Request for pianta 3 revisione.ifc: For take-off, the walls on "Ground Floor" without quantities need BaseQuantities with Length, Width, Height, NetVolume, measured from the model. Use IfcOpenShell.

First a look at what the model holds.

```python
import ifcopenshell
import ifcopenshell.util.element
import ifcopenshell.util.unit

model = ifcopenshell.open("pianta 3 revisione.ifc")
print(model.schema)
for unit_type in ("LENGTHUNIT", "AREAUNIT", "VOLUMEUNIT"):
    print(unit_type, ifcopenshell.util.unit.calculate_unit_scale(model, unit_type))
storey = next(s for s in model.by_type("IfcBuildingStorey") if s.Name == "Ground Floor")
walls = [e for e in ifcopenshell.util.element.get_decomposition(storey) if e.is_a("IfcWall")]
for e in sorted(walls, key=lambda e: e.id()):
    print(e.id(), e.is_a(), e.Name, list(ifcopenshell.util.element.get_psets(e, qtos_only=True)), sep=" | ")
```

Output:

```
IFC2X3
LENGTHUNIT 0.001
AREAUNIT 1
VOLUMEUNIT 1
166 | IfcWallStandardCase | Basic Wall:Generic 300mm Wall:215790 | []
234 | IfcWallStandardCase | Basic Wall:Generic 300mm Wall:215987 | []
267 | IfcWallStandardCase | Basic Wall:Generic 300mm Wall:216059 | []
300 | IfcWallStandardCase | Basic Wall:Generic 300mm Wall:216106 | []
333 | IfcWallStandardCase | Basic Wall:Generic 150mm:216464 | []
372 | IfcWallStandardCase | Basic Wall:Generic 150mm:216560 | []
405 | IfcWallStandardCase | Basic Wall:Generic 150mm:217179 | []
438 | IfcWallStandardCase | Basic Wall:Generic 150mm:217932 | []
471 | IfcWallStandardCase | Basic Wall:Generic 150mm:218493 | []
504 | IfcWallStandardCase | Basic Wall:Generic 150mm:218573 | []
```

```python
import ifcopenshell
import ifcopenshell.api.pset
import ifcopenshell.geom
import ifcopenshell.util.element
import ifcopenshell.util.shape
import ifcopenshell.util.unit

model = ifcopenshell.open("pianta 3 revisione.ifc")
unit_scale = ifcopenshell.util.unit.calculate_unit_scale(model)
volume_scale = ifcopenshell.util.unit.calculate_unit_scale(model, "VOLUMEUNIT")
settings = ifcopenshell.geom.settings()

storey = next(s for s in model.by_type("IfcBuildingStorey") if s.Name == "Ground Floor")
walls = [e for e in ifcopenshell.util.element.get_decomposition(storey) if e.is_a("IfcWall")]

for e in sorted(walls, key=lambda e: e.id()):
    if ifcopenshell.util.element.get_psets(e, qtos_only=True, should_inherit=False):
        continue
    # Geometry comes back in metres, in the element's own axes.
    shape = ifcopenshell.geom.create_shape(settings, e)
    values = {
        "Length": ifcopenshell.util.shape.get_x(shape.geometry) / unit_scale,
        "Width": ifcopenshell.util.shape.get_y(shape.geometry) / unit_scale,
        "Height": ifcopenshell.util.shape.get_z(shape.geometry) / unit_scale,
        "NetVolume": ifcopenshell.util.shape.get_volume(shape.geometry) / volume_scale,
    }
    qto = ifcopenshell.api.pset.add_qto(model, product=e, name="BaseQuantities")
    ifcopenshell.api.pset.edit_qto(model, qto=qto, properties=values)
    print(e.id(), {k: round(v, 3) for k, v in values.items()})

model.write("pianta 3 revisione_v2.ifc")
```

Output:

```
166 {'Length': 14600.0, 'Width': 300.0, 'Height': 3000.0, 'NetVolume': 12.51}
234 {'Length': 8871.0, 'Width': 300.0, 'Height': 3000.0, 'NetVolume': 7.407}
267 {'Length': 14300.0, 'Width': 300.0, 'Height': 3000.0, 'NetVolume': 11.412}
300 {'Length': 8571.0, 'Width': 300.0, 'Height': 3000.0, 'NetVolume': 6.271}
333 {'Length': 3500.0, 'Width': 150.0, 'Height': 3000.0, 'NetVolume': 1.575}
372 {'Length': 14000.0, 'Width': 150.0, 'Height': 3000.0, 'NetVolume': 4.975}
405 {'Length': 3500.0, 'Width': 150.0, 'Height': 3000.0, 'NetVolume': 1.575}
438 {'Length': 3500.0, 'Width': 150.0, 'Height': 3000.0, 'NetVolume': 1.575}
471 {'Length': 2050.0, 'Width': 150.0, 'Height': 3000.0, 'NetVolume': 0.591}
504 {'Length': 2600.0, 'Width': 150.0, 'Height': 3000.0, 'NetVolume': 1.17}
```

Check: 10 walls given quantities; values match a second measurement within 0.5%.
